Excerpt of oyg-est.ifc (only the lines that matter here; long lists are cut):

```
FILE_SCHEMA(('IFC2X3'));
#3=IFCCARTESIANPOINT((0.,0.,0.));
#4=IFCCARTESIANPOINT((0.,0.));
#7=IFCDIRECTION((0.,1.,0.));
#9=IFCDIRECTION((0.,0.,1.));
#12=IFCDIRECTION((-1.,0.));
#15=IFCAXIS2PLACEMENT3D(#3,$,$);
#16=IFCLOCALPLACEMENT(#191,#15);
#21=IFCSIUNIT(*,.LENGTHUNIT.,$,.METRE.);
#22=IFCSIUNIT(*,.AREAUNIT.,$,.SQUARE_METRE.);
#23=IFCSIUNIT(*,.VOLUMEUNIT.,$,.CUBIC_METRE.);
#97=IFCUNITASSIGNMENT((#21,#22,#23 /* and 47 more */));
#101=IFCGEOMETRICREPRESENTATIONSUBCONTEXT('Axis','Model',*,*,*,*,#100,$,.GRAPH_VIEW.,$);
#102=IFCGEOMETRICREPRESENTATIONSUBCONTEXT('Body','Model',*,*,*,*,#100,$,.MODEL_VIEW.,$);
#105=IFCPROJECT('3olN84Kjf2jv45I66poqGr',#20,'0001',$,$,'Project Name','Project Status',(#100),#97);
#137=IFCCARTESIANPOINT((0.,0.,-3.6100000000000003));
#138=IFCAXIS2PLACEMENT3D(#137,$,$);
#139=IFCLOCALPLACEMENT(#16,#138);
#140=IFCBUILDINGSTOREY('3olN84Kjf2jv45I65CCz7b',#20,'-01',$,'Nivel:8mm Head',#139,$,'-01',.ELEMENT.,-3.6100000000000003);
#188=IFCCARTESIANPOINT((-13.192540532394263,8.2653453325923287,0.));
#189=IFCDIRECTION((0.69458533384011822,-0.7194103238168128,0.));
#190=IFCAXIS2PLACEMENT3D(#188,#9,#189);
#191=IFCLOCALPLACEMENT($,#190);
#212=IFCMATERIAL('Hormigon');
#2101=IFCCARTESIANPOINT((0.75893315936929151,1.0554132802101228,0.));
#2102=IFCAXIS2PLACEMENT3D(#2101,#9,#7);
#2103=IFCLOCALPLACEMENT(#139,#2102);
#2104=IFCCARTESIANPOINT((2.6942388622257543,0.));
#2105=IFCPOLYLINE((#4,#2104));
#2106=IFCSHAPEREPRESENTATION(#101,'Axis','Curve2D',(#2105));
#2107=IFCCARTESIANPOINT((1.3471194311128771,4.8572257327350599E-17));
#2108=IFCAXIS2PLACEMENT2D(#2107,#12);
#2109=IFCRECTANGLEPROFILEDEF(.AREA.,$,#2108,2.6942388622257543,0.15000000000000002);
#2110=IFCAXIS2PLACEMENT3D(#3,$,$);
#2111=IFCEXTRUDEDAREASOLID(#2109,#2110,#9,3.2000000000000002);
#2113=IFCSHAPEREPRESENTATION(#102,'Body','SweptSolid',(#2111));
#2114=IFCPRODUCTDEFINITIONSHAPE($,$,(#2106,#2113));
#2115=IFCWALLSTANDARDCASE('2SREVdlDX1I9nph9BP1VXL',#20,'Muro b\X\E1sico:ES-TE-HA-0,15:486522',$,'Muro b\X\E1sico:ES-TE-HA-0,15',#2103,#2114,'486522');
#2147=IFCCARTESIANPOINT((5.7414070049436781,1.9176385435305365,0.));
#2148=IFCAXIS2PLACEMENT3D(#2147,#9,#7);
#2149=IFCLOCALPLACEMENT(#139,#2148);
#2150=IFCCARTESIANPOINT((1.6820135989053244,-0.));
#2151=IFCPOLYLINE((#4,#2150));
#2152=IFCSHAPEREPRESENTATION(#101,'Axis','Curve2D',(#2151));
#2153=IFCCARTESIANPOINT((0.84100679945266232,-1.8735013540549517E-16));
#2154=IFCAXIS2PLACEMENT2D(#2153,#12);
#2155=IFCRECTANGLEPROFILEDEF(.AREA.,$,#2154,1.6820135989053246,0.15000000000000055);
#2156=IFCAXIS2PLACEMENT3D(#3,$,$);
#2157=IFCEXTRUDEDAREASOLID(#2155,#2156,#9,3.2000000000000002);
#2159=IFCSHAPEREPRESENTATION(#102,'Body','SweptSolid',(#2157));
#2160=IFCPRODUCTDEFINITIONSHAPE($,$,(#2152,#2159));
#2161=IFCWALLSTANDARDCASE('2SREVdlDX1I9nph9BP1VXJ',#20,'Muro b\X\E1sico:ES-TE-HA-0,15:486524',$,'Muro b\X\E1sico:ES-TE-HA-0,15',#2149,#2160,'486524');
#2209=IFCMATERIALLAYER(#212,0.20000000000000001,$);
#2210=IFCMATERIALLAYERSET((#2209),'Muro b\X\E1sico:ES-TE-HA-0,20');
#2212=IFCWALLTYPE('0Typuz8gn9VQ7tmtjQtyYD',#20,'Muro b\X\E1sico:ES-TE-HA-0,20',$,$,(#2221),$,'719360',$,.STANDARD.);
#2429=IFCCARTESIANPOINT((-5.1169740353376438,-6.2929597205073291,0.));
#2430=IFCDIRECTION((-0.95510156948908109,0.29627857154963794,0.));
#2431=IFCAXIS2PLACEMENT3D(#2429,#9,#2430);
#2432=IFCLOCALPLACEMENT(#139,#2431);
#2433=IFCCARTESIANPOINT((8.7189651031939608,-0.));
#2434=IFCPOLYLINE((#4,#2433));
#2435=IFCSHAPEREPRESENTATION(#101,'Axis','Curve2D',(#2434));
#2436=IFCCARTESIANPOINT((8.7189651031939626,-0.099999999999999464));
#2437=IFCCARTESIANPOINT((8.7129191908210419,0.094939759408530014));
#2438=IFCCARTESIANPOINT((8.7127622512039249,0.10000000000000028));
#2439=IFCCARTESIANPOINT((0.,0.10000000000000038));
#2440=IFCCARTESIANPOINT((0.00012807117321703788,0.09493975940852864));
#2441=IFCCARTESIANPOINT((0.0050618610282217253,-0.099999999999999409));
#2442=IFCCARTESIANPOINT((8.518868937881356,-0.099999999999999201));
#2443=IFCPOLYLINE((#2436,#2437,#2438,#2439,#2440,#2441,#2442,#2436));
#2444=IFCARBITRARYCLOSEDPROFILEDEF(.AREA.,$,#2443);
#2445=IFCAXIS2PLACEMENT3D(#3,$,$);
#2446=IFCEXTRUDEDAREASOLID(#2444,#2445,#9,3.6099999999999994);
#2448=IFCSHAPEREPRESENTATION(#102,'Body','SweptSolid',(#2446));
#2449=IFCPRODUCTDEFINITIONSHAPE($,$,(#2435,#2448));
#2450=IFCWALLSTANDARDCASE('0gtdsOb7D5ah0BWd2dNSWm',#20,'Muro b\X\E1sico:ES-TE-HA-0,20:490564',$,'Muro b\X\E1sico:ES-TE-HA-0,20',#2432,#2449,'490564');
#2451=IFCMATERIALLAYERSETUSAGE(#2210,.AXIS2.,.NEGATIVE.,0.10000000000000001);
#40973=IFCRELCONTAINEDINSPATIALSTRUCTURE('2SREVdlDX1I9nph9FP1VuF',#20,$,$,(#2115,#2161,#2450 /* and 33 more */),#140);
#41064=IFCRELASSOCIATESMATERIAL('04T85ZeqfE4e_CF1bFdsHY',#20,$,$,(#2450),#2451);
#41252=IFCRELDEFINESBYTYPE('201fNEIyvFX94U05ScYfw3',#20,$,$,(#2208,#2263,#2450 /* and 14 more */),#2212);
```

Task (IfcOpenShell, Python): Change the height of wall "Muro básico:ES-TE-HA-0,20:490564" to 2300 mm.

```python
import ifcopenshell
import ifcopenshell.geom
import ifcopenshell.util.representation
import ifcopenshell.util.shape
import ifcopenshell.util.unit

model = ifcopenshell.open("oyg-est.ifc")
unit_scale = ifcopenshell.util.unit.calculate_unit_scale(model)
settings = ifcopenshell.geom.settings()


def volume(element):
    """Net volume in cubic metres, openings subtracted."""
    shape = ifcopenshell.geom.create_shape(settings, element)
    return ifcopenshell.util.shape.get_volume(shape.geometry)


wall = model.by_id(2450)
before = volume(wall)

body = ifcopenshell.util.representation.get_representation(wall, "Model", "Body")
solid = body.Items[0]
old_height = solid.Depth
solid.Depth = 2.3 / unit_scale
after = volume(wall)

print(f"height {old_height:g} -> {solid.Depth:g}, volume {before:.3f} -> {after:.3f} m3")

model.write("oyg-est_rev.ifc")
```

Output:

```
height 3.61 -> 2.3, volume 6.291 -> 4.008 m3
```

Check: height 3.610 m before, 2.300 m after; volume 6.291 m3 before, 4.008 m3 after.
